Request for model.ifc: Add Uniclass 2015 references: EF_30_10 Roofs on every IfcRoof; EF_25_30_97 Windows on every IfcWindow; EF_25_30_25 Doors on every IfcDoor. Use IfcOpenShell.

First a look at what the model holds.

```python
import ifcopenshell

model = ifcopenshell.open("model.ifc")
print(model.schema)
print("classifications:", [c.Name for c in model.by_type("IfcClassification")])
for ifc_class in ("IfcDoor", "IfcRoof", "IfcStair", "IfcWall", "IfcWindow"):
    print(ifc_class, len(model.by_type(ifc_class)))
```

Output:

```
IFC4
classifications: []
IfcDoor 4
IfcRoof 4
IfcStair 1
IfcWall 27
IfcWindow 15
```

```python
import ifcopenshell
import ifcopenshell.api.classification

model = ifcopenshell.open("model.ifc")

system = ifcopenshell.api.classification.add_classification(model, classification="Uniclass 2015")

codes = {
    "IfcRoof": ("EF_30_10", "Roofs"),
    "IfcWindow": ("EF_25_30_97", "Windows"),
    "IfcDoor": ("EF_25_30_25", "Doors"),
}
for ifc_class, (code, name) in codes.items():
    products = model.by_type(ifc_class)
    ifcopenshell.api.classification.add_reference(
        model, products=products, classification=system, identification=code, name=name
    )
    print(code, len(products))

model.write("model_edited.ifc")
```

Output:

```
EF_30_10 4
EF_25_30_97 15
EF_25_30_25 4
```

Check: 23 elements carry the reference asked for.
